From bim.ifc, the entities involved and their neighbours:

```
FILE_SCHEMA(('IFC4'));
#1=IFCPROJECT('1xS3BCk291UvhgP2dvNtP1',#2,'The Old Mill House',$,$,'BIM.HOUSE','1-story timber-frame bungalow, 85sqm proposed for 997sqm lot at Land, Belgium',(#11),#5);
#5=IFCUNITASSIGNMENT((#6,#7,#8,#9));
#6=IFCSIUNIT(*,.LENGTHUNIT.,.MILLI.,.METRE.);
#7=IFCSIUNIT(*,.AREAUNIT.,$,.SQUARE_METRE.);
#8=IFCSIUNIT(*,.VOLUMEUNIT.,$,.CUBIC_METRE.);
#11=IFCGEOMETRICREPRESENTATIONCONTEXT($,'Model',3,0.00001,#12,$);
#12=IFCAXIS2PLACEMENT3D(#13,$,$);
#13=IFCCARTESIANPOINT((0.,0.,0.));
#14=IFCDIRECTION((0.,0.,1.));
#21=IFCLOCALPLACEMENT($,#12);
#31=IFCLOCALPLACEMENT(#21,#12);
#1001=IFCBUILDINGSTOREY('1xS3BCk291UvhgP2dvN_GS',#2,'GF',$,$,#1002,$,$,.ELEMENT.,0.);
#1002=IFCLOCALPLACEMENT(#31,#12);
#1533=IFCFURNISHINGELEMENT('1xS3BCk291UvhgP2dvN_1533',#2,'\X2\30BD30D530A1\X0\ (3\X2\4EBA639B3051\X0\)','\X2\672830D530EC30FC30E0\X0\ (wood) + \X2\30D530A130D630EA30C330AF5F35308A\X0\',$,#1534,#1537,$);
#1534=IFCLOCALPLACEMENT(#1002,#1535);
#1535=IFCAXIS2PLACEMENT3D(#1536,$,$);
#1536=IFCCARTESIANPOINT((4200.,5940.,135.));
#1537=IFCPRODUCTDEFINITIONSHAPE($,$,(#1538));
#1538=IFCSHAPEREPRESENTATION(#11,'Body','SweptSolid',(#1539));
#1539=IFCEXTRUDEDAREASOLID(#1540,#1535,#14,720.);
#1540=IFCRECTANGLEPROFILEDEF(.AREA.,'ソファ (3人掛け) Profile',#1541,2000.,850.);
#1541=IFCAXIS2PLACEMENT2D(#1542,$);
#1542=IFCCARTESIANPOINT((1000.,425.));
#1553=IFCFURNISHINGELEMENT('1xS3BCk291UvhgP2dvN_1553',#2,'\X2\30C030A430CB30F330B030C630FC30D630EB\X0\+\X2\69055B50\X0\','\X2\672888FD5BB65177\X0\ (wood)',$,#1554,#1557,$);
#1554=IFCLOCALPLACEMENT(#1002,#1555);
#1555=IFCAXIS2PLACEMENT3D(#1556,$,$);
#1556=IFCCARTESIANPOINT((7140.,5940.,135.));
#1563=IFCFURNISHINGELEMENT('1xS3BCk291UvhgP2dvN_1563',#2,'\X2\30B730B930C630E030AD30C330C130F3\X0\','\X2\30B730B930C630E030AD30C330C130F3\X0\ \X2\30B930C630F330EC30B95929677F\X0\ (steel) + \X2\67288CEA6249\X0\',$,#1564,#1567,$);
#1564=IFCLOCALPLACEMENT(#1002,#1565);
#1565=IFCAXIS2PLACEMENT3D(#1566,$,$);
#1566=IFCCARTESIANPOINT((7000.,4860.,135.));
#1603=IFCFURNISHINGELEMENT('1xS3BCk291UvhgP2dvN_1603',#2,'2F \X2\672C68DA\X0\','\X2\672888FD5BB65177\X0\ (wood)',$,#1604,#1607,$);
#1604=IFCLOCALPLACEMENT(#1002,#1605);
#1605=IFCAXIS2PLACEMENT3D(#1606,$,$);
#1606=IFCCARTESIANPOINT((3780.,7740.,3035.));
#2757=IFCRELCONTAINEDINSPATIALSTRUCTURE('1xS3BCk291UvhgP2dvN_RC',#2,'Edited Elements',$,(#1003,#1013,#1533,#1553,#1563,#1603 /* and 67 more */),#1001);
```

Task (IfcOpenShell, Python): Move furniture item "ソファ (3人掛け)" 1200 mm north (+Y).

```python
import ifcopenshell
import ifcopenshell.api.geometry
import ifcopenshell.util.placement

model = ifcopenshell.open("bim.ifc")

item = model.by_id(1533)
matrix = ifcopenshell.util.placement.get_local_placement(item.ObjectPlacement)
matrix[1, 3] += 1200.0
ifcopenshell.api.geometry.edit_object_placement(model, product=item, matrix=matrix, is_si=False)

print(ifcopenshell.util.placement.get_local_placement(item.ObjectPlacement).round(3) + 0.0)

model.write("bim_v2.ifc")
```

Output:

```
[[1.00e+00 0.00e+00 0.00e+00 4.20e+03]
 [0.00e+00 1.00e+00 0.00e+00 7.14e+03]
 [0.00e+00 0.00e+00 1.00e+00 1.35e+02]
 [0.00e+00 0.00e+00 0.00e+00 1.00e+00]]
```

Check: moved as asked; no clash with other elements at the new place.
